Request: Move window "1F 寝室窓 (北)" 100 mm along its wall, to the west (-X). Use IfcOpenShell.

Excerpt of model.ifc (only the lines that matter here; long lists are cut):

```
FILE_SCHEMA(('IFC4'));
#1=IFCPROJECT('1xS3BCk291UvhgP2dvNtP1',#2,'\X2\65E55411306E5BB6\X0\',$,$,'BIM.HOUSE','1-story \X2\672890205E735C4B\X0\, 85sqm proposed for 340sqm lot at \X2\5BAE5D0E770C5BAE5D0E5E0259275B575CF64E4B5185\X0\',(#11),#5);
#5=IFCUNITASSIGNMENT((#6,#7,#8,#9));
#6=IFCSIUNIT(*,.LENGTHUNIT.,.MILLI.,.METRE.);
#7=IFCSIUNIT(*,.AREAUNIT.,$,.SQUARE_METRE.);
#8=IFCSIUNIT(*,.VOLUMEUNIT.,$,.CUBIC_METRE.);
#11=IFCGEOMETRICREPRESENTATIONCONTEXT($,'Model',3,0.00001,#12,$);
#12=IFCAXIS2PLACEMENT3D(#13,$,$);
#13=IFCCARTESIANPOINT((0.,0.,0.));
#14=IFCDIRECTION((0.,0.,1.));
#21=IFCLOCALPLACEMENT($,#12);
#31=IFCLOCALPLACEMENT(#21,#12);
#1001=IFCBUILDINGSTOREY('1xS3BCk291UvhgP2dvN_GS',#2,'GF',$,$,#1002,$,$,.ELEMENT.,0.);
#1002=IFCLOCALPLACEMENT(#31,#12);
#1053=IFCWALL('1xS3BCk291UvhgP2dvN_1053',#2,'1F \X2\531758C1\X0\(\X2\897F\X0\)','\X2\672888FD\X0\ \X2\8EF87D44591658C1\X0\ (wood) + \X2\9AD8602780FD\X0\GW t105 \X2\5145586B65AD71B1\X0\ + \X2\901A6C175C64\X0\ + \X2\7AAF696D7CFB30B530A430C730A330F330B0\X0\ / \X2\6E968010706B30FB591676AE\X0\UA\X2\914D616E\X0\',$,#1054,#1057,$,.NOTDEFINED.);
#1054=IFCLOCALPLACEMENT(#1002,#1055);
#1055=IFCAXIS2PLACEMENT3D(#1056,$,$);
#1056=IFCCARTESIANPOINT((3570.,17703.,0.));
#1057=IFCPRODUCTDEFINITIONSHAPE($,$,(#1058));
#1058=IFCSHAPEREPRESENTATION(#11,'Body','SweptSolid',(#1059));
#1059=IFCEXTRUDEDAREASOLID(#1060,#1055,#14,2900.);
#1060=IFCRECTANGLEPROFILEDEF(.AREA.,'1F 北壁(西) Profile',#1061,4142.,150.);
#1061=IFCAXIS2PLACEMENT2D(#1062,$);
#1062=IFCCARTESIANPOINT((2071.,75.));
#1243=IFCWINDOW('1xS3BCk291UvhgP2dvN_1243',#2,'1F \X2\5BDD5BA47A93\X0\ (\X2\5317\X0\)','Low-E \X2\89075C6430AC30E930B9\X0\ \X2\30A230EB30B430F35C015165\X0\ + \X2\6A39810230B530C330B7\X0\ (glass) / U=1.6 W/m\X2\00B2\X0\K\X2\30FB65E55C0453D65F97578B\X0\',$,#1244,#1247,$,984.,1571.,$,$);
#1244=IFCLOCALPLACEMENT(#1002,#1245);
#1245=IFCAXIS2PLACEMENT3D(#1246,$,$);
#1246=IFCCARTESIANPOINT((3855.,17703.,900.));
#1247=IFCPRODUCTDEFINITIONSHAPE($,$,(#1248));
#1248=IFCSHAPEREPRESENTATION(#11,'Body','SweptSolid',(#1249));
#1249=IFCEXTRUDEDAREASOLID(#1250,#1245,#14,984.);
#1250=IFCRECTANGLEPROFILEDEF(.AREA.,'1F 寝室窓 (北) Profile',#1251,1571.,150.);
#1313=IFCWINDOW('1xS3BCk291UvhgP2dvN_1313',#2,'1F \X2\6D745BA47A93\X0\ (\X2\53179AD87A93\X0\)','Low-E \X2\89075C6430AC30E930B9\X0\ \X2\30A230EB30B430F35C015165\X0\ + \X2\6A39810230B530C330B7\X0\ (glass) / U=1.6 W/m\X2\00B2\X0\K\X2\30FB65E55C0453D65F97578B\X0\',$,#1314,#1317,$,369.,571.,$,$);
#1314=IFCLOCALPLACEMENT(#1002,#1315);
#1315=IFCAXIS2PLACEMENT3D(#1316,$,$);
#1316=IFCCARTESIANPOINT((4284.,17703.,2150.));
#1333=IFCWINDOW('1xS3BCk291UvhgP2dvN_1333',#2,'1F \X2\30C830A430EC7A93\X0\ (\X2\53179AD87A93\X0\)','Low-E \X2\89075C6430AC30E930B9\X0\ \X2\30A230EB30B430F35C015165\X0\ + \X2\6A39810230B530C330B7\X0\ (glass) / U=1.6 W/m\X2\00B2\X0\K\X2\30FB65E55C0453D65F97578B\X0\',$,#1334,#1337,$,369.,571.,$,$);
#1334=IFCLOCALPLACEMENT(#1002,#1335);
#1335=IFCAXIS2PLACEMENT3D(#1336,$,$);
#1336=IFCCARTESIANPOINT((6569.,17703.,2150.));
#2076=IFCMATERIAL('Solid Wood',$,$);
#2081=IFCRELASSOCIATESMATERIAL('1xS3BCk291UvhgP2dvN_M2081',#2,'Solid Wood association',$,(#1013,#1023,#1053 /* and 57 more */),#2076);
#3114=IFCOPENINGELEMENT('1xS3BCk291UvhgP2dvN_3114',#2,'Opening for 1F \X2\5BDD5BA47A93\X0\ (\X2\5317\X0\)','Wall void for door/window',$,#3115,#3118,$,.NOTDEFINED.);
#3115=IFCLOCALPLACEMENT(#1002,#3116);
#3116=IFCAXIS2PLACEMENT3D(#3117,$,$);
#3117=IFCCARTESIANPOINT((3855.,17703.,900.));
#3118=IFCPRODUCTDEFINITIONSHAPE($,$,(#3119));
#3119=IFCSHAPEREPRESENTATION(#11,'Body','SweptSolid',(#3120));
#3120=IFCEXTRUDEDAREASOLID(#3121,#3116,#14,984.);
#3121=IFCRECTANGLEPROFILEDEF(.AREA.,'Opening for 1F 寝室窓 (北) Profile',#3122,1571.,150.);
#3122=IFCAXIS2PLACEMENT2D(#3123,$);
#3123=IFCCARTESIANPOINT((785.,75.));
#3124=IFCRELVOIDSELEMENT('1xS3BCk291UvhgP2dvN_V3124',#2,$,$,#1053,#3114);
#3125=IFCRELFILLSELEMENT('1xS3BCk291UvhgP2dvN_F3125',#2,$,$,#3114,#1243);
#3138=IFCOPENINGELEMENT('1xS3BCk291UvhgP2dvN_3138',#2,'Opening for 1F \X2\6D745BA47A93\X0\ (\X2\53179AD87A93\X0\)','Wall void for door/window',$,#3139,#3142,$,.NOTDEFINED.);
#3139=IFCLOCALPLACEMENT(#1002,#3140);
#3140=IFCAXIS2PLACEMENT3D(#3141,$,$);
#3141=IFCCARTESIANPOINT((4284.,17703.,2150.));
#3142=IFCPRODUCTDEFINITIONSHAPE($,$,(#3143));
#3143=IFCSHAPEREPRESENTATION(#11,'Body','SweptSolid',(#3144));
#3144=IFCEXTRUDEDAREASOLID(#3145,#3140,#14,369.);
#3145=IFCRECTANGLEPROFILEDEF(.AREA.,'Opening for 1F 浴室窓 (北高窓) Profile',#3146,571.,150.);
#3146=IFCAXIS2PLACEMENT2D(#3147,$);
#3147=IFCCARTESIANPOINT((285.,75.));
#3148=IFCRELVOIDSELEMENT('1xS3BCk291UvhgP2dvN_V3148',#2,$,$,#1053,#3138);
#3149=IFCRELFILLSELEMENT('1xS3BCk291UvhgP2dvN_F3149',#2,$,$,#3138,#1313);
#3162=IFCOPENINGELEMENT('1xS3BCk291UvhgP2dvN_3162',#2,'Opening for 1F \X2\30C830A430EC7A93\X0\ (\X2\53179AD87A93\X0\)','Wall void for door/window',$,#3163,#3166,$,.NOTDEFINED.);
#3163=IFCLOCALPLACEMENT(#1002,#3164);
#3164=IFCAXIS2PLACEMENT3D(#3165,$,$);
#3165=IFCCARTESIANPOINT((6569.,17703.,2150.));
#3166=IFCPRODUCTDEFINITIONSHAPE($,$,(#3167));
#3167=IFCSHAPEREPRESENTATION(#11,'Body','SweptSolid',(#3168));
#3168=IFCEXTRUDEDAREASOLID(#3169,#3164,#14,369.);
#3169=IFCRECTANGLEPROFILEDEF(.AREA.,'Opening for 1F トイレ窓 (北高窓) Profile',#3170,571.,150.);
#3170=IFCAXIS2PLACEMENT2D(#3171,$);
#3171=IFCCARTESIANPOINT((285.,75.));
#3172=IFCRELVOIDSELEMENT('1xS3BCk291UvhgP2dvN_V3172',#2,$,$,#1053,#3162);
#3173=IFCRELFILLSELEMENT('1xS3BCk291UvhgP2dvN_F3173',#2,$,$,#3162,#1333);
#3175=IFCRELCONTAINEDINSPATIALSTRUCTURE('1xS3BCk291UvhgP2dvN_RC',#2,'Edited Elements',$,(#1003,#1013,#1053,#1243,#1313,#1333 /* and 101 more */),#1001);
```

```python
import ifcopenshell
import ifcopenshell.api.geometry
import ifcopenshell.util.placement

model = ifcopenshell.open("model.ifc")

window = model.by_id(1243)
opening = window.FillsVoids[0].RelatingOpeningElement
wall = opening.VoidsElements[0].RelatingBuildingElement

wall_matrix = ifcopenshell.util.placement.get_local_placement(wall.ObjectPlacement)
shift = wall_matrix[:3, 0] * -100.0
before = ifcopenshell.util.placement.get_local_placement(window.ObjectPlacement)[:3, 3].copy()

# The window is not placed relative to its opening, so move both.
for product in (opening, window):
    matrix = ifcopenshell.util.placement.get_local_placement(product.ObjectPlacement)
    matrix[:3, 3] += shift
    ifcopenshell.api.geometry.edit_object_placement(model, product=product, matrix=matrix, is_si=False)

after = ifcopenshell.util.placement.get_local_placement(window.ObjectPlacement)[:3, 3]
print("window moved by", (after - before).round(3) + 0.0)

model.write("model_edited.ifc")
```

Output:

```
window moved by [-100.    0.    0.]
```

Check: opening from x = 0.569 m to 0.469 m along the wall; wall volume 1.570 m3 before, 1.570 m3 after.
